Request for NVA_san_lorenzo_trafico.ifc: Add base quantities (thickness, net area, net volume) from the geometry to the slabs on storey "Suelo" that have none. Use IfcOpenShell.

First a look at what the model holds.

```python
import ifcopenshell
import ifcopenshell.util.element
import ifcopenshell.util.unit

model = ifcopenshell.open("NVA_san_lorenzo_trafico.ifc")
print(model.schema)
for unit_type in ("LENGTHUNIT", "AREAUNIT", "VOLUMEUNIT"):
    print(unit_type, ifcopenshell.util.unit.calculate_unit_scale(model, unit_type))
storey = next(s for s in model.by_type("IfcBuildingStorey") if s.Name == "Suelo")
slabs = [e for e in ifcopenshell.util.element.get_decomposition(storey) if e.is_a("IfcSlab")]
for e in sorted(slabs, key=lambda e: e.id()):
    print(e.id(), e.is_a(), e.Name, list(ifcopenshell.util.element.get_psets(e, qtos_only=True)), sep=" | ")
```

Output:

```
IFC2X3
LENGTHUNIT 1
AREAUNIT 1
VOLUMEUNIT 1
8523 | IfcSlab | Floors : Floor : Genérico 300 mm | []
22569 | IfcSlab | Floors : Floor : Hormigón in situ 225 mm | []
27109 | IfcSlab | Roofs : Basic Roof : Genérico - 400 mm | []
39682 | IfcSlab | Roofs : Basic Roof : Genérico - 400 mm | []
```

```python
import ifcopenshell
import ifcopenshell.api.pset
import ifcopenshell.geom
import ifcopenshell.util.element
import ifcopenshell.util.shape
import ifcopenshell.util.unit

model = ifcopenshell.open("NVA_san_lorenzo_trafico.ifc")
unit_scale = ifcopenshell.util.unit.calculate_unit_scale(model)
area_scale = ifcopenshell.util.unit.calculate_unit_scale(model, "AREAUNIT")
volume_scale = ifcopenshell.util.unit.calculate_unit_scale(model, "VOLUMEUNIT")
settings = ifcopenshell.geom.settings()

storey = next(s for s in model.by_type("IfcBuildingStorey") if s.Name == "Suelo")
slabs = [e for e in ifcopenshell.util.element.get_decomposition(storey) if e.is_a("IfcSlab")]

for e in sorted(slabs, key=lambda e: e.id()):
    if ifcopenshell.util.element.get_psets(e, qtos_only=True, should_inherit=False):
        continue
    # Geometry comes back in metres, in the element's own axes.
    shape = ifcopenshell.geom.create_shape(settings, e)
    values = {
        "Width": ifcopenshell.util.shape.get_z(shape.geometry) / unit_scale,
        "NetArea": ifcopenshell.util.shape.get_footprint_area(shape.geometry) / area_scale,
        "NetVolume": ifcopenshell.util.shape.get_volume(shape.geometry) / volume_scale,
    }
    qto = ifcopenshell.api.pset.add_qto(model, product=e, name="BaseQuantities")
    ifcopenshell.api.pset.edit_qto(model, qto=qto, properties=values)
    print(e.id(), {k: round(v, 3) for k, v in values.items()})

model.write("NVA_san_lorenzo_trafico_updated.ifc")
```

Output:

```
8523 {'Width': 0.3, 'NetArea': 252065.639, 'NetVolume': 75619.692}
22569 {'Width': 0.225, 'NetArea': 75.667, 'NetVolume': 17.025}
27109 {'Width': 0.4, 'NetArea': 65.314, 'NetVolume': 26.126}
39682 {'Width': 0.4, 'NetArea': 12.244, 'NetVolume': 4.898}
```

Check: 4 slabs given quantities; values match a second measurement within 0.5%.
